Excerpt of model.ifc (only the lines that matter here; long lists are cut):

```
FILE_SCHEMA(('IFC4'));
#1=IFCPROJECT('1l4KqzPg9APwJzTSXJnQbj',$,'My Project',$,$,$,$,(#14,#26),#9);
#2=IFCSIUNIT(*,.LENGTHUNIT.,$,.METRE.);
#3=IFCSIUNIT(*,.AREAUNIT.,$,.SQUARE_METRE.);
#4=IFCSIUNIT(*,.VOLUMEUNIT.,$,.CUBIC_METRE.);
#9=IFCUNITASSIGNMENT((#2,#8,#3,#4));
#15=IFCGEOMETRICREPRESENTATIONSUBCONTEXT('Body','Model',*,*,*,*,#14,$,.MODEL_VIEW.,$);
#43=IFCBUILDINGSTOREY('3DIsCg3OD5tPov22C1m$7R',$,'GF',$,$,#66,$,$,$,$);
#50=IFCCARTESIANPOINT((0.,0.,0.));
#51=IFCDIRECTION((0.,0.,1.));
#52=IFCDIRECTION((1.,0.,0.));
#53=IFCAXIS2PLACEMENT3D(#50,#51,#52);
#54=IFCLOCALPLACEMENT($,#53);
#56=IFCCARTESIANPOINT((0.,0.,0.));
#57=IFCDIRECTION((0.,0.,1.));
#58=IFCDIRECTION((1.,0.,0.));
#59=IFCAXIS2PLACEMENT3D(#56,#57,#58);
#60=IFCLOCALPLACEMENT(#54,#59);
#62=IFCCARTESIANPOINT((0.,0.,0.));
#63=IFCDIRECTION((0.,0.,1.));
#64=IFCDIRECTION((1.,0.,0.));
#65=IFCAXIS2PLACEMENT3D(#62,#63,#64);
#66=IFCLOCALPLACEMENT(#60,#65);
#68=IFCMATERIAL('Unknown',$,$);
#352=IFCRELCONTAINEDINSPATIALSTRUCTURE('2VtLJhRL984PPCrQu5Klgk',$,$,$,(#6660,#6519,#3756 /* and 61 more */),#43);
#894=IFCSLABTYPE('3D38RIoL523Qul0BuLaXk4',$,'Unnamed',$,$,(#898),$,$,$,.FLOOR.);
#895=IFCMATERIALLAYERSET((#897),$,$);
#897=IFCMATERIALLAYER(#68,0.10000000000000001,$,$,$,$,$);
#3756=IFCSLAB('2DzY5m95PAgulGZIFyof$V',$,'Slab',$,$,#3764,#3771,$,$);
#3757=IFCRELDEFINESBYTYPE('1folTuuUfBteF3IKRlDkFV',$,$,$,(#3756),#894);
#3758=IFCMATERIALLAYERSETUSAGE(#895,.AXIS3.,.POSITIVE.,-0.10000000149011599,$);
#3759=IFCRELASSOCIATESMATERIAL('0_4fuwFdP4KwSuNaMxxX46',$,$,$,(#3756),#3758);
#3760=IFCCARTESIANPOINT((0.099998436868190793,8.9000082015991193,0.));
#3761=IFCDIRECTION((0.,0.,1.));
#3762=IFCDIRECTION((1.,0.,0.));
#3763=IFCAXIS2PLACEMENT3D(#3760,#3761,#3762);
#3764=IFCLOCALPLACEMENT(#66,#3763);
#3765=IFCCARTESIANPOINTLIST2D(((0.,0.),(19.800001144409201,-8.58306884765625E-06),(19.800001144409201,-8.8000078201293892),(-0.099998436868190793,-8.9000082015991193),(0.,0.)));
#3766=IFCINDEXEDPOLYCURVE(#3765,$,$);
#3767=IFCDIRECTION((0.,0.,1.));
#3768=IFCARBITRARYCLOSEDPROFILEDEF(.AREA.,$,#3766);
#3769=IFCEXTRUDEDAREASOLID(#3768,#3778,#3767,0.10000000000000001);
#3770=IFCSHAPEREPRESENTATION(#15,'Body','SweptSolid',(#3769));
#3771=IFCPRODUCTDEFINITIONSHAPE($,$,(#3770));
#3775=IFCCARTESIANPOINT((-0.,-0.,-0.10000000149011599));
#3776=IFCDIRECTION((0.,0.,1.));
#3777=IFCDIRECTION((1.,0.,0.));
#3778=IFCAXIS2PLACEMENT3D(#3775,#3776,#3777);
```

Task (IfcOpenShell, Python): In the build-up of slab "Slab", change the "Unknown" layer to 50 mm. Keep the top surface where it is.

```python
import ifcopenshell
import ifcopenshell.util.element
import ifcopenshell.util.representation
import ifcopenshell.util.unit

model = ifcopenshell.open("model.ifc")
unit_scale = ifcopenshell.util.unit.calculate_unit_scale(model)

layer_set = model.by_id(895)
layer = next(l for l in layer_set.MaterialLayers if l.Material and l.Material.Name == "Unknown")
change = 0.05 / unit_scale - layer.LayerThickness
layer.LayerThickness += change

# Geometry does not follow the layer set by itself.
slabs = [e for e in ifcopenshell.util.element.get_elements_by_material(model, layer_set) if e.is_a("IfcSlab")]
for slab in sorted(slabs, key=lambda e: e.id()):
    body = ifcopenshell.util.representation.get_representation(slab, "Model", "Body")
    solid = body.Items[0]
    old_depth = solid.Depth
    solid.Depth += change
    # Extruded upwards: lower the start of the extrusion so the top stays.
    x, y, z = solid.Position.Location.Coordinates
    solid.Position.Location = model.createIfcCartesianPoint((x, y, z - change))
    print(slab.id(), f"{old_depth:g} -> {solid.Depth:g}")

# The layers are counted up from the underside, which has moved.
for usage in {ifcopenshell.util.element.get_material(slab) for slab in slabs}:
    usage.OffsetFromReferenceLine -= change

model.write("model_v2.ifc")
```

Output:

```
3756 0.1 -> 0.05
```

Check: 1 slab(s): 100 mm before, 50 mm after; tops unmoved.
